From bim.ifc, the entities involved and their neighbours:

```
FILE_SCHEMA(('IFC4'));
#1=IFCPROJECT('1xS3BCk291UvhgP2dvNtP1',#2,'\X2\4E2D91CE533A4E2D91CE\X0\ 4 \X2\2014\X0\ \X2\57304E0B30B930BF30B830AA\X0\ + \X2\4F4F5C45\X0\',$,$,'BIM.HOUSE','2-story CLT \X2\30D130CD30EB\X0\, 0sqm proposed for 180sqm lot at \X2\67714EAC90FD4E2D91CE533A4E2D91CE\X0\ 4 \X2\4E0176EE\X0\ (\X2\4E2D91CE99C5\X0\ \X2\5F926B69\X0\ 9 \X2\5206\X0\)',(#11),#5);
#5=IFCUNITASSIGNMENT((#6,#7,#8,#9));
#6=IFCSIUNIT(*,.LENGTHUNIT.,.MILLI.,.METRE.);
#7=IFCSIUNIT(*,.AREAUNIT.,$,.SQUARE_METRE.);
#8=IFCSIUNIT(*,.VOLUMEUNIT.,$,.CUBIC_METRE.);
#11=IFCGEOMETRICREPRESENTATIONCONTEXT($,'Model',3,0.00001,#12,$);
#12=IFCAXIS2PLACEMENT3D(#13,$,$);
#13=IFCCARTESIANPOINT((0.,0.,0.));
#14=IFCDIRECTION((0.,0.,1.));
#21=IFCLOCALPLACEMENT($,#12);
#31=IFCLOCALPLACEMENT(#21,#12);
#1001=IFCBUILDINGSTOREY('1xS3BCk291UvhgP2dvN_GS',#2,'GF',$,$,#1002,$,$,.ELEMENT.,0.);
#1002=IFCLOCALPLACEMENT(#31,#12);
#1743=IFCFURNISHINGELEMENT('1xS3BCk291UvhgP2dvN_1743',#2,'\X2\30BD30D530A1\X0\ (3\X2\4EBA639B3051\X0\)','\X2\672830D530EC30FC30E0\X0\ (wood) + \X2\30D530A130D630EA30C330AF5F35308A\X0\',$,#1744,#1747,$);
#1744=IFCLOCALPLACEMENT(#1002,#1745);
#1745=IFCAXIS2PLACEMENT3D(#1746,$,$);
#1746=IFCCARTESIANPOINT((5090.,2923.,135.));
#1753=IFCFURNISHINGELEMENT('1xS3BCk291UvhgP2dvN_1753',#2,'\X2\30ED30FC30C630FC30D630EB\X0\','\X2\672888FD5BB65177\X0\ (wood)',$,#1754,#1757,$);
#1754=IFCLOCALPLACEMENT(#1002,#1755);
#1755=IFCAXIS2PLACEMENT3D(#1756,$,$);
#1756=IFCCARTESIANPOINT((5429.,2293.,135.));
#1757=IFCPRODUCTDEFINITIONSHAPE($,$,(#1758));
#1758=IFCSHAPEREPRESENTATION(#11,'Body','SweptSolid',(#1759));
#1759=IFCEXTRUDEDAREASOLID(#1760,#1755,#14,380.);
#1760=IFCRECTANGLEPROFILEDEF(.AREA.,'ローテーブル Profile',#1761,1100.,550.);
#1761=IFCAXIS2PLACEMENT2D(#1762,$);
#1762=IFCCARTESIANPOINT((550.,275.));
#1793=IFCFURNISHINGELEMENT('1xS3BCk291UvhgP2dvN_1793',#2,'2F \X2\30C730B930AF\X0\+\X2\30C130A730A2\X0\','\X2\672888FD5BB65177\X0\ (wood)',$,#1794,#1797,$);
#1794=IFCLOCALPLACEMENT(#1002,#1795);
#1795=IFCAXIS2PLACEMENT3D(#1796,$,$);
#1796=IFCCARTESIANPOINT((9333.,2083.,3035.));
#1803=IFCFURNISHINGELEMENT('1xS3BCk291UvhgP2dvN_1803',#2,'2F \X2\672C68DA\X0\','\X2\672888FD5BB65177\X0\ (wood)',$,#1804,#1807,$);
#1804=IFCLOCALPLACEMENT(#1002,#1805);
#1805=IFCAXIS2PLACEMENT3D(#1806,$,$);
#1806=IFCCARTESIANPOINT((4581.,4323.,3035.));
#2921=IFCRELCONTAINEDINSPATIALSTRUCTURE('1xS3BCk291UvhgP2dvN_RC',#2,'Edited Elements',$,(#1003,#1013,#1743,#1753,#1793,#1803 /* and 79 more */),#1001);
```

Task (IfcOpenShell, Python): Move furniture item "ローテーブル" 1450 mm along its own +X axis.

```python
import ifcopenshell
import ifcopenshell.api.geometry
import ifcopenshell.util.placement
import ifcopenshell.util.unit

model = ifcopenshell.open("bim.ifc")
unit_scale = ifcopenshell.util.unit.calculate_unit_scale(model)

item = model.by_guid("1xS3BCk291UvhgP2dvN_1753")
matrix = ifcopenshell.util.placement.get_local_placement(item.ObjectPlacement)
matrix[:3, 3] += matrix[:3, 0] * 1.45 / unit_scale
ifcopenshell.api.geometry.edit_object_placement(model, product=item, matrix=matrix, is_si=False)

print(ifcopenshell.util.placement.get_local_placement(item.ObjectPlacement).round(3) + 0.0)

model.write("bim_v2.ifc")
```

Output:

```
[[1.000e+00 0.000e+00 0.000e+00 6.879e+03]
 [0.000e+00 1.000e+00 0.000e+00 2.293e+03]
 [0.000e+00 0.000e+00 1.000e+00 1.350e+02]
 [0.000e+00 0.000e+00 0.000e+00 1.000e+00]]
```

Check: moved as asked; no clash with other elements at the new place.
